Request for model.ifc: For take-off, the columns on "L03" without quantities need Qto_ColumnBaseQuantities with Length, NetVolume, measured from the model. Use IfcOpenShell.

First a look at what the model holds.

```python
import ifcopenshell
import ifcopenshell.util.element
import ifcopenshell.util.unit

model = ifcopenshell.open("model.ifc")
print(model.schema)
for unit_type in ("LENGTHUNIT", "AREAUNIT", "VOLUMEUNIT"):
    print(unit_type, ifcopenshell.util.unit.calculate_unit_scale(model, unit_type))
storey = next(s for s in model.by_type("IfcBuildingStorey") if s.Name == "L03")
columns = [e for e in ifcopenshell.util.element.get_decomposition(storey) if e.is_a("IfcColumn")]
for e in sorted(columns, key=lambda e: e.id()):
    print(e.id(), e.is_a(), e.Name, list(ifcopenshell.util.element.get_psets(e, qtos_only=True)), sep=" | ")
```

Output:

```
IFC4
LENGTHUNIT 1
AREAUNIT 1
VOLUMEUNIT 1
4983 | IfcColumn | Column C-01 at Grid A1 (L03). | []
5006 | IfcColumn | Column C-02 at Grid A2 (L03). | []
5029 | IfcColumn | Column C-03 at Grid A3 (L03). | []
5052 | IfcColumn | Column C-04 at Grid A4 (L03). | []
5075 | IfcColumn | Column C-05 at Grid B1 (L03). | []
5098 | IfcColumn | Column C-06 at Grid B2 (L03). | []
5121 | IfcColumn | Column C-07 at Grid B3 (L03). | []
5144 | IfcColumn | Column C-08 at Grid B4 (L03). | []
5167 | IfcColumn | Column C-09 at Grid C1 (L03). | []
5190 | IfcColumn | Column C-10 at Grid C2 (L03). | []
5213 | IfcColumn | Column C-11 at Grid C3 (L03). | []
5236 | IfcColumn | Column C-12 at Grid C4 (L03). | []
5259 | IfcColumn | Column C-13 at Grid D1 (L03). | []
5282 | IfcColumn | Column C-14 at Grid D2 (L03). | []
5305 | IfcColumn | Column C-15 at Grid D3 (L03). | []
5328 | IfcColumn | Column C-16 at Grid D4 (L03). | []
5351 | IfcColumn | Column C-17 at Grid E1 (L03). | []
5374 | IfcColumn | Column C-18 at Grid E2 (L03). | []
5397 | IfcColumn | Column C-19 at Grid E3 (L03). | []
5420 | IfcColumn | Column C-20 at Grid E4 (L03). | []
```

```python
import ifcopenshell
import ifcopenshell.api.pset
import ifcopenshell.geom
import ifcopenshell.util.element
import ifcopenshell.util.shape
import ifcopenshell.util.unit

model = ifcopenshell.open("model.ifc")
unit_scale = ifcopenshell.util.unit.calculate_unit_scale(model)
volume_scale = ifcopenshell.util.unit.calculate_unit_scale(model, "VOLUMEUNIT")
settings = ifcopenshell.geom.settings()

storey = next(s for s in model.by_type("IfcBuildingStorey") if s.Name == "L03")
columns = [e for e in ifcopenshell.util.element.get_decomposition(storey) if e.is_a("IfcColumn")]

for e in sorted(columns, key=lambda e: e.id()):
    if ifcopenshell.util.element.get_psets(e, qtos_only=True, should_inherit=False):
        continue
    # Geometry comes back in metres, in the element's own axes.
    shape = ifcopenshell.geom.create_shape(settings, e)
    values = {
        "Length": ifcopenshell.util.shape.get_z(shape.geometry) / unit_scale,
        "NetVolume": ifcopenshell.util.shape.get_volume(shape.geometry) / volume_scale,
    }
    qto = ifcopenshell.api.pset.add_qto(model, product=e, name="Qto_ColumnBaseQuantities")
    ifcopenshell.api.pset.edit_qto(model, qto=qto, properties=values)
    print(e.id(), {k: round(v, 3) for k, v in values.items()})

model.write("model-out.ifc")
```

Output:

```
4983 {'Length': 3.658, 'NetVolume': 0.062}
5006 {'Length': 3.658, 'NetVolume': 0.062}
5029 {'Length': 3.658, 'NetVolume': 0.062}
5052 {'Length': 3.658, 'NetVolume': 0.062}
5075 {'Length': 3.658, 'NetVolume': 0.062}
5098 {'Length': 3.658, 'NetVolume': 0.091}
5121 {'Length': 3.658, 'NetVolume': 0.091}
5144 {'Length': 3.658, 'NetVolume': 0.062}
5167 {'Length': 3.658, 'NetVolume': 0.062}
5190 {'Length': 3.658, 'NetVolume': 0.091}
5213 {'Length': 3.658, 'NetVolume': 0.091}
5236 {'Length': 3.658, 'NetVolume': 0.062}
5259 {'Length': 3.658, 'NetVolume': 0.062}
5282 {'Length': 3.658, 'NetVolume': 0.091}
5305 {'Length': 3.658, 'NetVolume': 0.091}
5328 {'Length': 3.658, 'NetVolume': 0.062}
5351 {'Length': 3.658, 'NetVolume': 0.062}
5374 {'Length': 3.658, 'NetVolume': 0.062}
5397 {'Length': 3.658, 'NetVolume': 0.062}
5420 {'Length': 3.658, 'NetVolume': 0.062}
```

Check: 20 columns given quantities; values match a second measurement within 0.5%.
